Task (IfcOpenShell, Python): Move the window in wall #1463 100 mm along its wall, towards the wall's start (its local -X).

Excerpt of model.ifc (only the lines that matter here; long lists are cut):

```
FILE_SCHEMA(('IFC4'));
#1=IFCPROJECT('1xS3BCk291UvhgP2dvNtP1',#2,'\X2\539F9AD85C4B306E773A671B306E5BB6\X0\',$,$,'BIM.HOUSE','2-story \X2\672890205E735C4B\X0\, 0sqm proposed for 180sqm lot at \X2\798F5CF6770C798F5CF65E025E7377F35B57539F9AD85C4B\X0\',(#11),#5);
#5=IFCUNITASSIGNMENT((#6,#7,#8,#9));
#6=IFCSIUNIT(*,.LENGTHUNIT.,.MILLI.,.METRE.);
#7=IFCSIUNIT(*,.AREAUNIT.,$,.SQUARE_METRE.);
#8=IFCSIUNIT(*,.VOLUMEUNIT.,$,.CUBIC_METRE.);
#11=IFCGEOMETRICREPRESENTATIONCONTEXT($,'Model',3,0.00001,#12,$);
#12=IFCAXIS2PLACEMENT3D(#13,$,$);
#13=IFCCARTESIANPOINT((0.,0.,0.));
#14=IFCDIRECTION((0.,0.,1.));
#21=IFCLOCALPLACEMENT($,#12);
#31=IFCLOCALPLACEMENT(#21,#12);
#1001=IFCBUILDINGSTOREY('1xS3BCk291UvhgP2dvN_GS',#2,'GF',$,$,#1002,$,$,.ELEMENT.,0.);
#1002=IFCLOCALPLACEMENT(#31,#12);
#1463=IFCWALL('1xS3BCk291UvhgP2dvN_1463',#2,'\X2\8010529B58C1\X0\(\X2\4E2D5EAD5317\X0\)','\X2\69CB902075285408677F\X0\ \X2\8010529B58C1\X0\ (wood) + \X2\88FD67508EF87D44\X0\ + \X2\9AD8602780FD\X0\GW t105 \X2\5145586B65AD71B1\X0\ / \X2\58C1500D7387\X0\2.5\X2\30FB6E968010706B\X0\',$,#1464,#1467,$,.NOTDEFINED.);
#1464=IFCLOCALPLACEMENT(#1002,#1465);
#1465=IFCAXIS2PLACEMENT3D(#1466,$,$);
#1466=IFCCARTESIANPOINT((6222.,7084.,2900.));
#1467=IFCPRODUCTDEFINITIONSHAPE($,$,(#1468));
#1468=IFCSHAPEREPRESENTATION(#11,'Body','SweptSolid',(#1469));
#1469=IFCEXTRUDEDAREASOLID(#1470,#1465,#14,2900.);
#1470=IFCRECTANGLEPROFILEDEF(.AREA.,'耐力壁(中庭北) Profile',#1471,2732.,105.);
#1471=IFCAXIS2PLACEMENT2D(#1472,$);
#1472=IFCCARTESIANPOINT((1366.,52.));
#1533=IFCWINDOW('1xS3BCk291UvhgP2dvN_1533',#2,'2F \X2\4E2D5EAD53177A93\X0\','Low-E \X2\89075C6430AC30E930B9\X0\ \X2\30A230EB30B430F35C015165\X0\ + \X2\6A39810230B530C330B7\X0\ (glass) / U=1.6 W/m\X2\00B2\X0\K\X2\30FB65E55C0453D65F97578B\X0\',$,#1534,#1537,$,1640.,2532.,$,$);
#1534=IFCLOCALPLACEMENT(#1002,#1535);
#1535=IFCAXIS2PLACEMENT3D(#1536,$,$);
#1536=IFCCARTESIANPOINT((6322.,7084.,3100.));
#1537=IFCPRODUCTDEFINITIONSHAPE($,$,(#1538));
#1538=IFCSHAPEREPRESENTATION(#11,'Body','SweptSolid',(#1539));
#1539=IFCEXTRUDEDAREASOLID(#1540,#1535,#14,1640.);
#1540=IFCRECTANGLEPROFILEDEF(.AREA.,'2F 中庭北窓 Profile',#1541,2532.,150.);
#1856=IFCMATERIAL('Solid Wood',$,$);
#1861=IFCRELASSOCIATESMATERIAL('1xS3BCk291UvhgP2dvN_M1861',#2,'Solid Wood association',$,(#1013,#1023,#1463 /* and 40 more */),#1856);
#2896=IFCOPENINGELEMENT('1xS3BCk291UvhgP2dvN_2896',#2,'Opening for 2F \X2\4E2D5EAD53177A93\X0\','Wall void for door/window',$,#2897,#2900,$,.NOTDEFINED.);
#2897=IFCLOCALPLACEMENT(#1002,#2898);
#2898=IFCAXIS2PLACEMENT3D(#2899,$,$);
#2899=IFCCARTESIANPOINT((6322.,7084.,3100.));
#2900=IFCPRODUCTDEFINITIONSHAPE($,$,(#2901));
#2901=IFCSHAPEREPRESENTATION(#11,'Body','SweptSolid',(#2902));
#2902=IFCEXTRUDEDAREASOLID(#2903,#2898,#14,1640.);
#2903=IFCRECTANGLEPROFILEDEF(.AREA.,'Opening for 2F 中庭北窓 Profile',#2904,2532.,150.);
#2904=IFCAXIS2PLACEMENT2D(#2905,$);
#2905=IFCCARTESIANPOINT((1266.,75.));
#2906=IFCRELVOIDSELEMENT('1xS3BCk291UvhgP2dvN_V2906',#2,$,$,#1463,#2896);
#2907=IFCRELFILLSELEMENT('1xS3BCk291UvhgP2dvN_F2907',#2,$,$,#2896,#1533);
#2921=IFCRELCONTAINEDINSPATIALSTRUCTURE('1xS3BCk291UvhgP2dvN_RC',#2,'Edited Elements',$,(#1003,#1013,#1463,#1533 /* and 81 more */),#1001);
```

```python
import ifcopenshell
import ifcopenshell.api.geometry
import ifcopenshell.util.placement

model = ifcopenshell.open("model.ifc")

window = model.by_guid("1xS3BCk291UvhgP2dvN_1533")
opening = window.FillsVoids[0].RelatingOpeningElement
wall = opening.VoidsElements[0].RelatingBuildingElement

wall_matrix = ifcopenshell.util.placement.get_local_placement(wall.ObjectPlacement)
shift = wall_matrix[:3, 0] * -100.0
before = ifcopenshell.util.placement.get_local_placement(window.ObjectPlacement)[:3, 3].copy()

# The window is not placed relative to its opening, so move both.
for product in (opening, window):
    matrix = ifcopenshell.util.placement.get_local_placement(product.ObjectPlacement)
    matrix[:3, 3] += shift
    ifcopenshell.api.geometry.edit_object_placement(model, product=product, matrix=matrix, is_si=False)

after = ifcopenshell.util.placement.get_local_placement(window.ObjectPlacement)[:3, 3]
print("window moved by", (after - before).round(3) + 0.0)

model.write("model_v2.ifc")
```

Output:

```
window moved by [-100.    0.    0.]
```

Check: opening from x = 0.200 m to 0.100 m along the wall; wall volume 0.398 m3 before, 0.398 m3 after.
